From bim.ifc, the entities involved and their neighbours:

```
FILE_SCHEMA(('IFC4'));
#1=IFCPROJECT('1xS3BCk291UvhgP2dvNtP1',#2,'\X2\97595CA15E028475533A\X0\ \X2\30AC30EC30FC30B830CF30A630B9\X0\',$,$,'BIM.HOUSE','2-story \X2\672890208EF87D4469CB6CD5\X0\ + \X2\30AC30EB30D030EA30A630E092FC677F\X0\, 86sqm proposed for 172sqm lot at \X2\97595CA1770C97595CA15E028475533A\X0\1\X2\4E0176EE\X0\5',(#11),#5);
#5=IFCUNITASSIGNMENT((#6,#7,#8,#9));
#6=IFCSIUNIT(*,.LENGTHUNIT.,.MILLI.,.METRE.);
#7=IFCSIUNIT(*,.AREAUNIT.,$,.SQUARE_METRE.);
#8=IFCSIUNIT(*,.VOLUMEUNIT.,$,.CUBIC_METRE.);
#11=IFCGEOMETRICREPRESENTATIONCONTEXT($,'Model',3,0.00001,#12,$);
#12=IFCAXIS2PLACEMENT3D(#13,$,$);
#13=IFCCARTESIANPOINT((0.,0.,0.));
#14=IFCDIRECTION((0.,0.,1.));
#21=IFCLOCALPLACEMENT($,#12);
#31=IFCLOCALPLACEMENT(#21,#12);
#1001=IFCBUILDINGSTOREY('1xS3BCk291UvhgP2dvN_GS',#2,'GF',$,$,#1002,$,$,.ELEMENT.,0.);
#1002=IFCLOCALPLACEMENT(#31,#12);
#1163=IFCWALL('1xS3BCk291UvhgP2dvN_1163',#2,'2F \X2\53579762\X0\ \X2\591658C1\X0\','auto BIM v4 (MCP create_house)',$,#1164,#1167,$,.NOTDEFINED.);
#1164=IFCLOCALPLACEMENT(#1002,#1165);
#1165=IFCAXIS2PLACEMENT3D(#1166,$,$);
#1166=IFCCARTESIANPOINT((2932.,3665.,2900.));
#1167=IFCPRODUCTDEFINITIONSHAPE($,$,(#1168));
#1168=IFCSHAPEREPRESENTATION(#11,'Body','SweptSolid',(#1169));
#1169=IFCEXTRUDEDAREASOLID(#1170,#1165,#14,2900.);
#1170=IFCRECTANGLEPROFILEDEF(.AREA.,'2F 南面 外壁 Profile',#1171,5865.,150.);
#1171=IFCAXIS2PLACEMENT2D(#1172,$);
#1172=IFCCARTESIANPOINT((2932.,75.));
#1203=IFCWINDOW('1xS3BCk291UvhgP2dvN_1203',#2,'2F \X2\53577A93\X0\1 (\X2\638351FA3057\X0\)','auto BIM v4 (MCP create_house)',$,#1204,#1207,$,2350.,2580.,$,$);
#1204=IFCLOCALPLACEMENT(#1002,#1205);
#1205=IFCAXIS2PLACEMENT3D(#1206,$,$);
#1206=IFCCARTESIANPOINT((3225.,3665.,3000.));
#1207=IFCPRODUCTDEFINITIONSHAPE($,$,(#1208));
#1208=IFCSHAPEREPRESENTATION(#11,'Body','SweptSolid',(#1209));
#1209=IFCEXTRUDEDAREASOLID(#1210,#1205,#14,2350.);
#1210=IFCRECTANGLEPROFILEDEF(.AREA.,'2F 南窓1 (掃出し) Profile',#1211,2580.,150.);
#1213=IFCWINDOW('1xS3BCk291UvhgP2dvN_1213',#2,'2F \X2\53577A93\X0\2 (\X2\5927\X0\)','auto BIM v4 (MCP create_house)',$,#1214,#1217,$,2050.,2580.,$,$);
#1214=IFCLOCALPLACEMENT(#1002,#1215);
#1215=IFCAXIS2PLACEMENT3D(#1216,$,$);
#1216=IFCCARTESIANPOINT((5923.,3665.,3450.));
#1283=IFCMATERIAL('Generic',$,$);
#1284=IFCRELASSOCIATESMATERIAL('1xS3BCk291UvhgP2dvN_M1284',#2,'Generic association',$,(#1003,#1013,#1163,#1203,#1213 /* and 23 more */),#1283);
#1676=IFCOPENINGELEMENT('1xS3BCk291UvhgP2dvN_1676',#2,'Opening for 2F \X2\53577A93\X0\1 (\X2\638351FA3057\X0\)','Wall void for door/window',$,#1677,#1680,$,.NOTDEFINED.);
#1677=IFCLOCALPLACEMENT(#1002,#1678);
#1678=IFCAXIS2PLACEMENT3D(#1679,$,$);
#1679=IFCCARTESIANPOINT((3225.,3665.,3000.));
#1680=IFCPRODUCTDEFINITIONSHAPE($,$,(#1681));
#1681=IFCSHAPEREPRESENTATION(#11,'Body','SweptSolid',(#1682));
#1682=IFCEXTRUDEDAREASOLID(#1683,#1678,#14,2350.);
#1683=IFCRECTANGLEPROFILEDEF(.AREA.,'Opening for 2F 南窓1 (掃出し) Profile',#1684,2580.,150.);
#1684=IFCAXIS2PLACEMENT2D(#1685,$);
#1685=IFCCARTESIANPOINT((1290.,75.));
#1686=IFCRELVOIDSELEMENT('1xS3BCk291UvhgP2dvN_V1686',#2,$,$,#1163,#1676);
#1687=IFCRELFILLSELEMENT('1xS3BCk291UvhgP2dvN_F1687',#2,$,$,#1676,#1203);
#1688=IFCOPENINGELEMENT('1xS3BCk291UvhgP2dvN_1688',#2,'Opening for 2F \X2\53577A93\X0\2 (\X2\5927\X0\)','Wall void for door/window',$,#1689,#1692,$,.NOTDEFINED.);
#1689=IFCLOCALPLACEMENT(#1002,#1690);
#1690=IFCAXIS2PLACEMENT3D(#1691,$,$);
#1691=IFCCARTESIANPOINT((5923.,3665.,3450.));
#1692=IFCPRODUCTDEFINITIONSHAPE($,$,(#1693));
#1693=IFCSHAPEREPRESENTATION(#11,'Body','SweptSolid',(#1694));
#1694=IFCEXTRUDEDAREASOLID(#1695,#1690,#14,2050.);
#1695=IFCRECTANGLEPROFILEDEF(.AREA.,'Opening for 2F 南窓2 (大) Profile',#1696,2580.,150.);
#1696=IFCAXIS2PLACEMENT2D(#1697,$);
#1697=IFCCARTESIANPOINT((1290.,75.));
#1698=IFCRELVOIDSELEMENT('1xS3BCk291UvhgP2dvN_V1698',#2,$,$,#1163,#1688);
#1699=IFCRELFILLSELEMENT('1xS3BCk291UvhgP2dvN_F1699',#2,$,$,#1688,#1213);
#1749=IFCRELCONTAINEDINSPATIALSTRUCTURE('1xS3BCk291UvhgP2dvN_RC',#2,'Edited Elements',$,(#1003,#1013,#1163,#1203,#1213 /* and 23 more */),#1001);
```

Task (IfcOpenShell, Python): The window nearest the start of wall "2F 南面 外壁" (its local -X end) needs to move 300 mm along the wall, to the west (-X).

```python
import ifcopenshell
import ifcopenshell.api.geometry
import ifcopenshell.util.placement

model = ifcopenshell.open("bim.ifc")

window = model.by_guid("1xS3BCk291UvhgP2dvN_1203")
opening = window.FillsVoids[0].RelatingOpeningElement
wall = opening.VoidsElements[0].RelatingBuildingElement

wall_matrix = ifcopenshell.util.placement.get_local_placement(wall.ObjectPlacement)
shift = wall_matrix[:3, 0] * -300.0
before = ifcopenshell.util.placement.get_local_placement(window.ObjectPlacement)[:3, 3].copy()

# The window is not placed relative to its opening, so move both.
for product in (opening, window):
    matrix = ifcopenshell.util.placement.get_local_placement(product.ObjectPlacement)
    matrix[:3, 3] += shift
    ifcopenshell.api.geometry.edit_object_placement(model, product=product, matrix=matrix, is_si=False)

after = ifcopenshell.util.placement.get_local_placement(window.ObjectPlacement)[:3, 3]
print("window moved by", (after - before).round(3) + 0.0)

model.write("bim_v2.ifc")
```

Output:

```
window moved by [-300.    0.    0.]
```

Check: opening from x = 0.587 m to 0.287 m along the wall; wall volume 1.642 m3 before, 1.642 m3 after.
